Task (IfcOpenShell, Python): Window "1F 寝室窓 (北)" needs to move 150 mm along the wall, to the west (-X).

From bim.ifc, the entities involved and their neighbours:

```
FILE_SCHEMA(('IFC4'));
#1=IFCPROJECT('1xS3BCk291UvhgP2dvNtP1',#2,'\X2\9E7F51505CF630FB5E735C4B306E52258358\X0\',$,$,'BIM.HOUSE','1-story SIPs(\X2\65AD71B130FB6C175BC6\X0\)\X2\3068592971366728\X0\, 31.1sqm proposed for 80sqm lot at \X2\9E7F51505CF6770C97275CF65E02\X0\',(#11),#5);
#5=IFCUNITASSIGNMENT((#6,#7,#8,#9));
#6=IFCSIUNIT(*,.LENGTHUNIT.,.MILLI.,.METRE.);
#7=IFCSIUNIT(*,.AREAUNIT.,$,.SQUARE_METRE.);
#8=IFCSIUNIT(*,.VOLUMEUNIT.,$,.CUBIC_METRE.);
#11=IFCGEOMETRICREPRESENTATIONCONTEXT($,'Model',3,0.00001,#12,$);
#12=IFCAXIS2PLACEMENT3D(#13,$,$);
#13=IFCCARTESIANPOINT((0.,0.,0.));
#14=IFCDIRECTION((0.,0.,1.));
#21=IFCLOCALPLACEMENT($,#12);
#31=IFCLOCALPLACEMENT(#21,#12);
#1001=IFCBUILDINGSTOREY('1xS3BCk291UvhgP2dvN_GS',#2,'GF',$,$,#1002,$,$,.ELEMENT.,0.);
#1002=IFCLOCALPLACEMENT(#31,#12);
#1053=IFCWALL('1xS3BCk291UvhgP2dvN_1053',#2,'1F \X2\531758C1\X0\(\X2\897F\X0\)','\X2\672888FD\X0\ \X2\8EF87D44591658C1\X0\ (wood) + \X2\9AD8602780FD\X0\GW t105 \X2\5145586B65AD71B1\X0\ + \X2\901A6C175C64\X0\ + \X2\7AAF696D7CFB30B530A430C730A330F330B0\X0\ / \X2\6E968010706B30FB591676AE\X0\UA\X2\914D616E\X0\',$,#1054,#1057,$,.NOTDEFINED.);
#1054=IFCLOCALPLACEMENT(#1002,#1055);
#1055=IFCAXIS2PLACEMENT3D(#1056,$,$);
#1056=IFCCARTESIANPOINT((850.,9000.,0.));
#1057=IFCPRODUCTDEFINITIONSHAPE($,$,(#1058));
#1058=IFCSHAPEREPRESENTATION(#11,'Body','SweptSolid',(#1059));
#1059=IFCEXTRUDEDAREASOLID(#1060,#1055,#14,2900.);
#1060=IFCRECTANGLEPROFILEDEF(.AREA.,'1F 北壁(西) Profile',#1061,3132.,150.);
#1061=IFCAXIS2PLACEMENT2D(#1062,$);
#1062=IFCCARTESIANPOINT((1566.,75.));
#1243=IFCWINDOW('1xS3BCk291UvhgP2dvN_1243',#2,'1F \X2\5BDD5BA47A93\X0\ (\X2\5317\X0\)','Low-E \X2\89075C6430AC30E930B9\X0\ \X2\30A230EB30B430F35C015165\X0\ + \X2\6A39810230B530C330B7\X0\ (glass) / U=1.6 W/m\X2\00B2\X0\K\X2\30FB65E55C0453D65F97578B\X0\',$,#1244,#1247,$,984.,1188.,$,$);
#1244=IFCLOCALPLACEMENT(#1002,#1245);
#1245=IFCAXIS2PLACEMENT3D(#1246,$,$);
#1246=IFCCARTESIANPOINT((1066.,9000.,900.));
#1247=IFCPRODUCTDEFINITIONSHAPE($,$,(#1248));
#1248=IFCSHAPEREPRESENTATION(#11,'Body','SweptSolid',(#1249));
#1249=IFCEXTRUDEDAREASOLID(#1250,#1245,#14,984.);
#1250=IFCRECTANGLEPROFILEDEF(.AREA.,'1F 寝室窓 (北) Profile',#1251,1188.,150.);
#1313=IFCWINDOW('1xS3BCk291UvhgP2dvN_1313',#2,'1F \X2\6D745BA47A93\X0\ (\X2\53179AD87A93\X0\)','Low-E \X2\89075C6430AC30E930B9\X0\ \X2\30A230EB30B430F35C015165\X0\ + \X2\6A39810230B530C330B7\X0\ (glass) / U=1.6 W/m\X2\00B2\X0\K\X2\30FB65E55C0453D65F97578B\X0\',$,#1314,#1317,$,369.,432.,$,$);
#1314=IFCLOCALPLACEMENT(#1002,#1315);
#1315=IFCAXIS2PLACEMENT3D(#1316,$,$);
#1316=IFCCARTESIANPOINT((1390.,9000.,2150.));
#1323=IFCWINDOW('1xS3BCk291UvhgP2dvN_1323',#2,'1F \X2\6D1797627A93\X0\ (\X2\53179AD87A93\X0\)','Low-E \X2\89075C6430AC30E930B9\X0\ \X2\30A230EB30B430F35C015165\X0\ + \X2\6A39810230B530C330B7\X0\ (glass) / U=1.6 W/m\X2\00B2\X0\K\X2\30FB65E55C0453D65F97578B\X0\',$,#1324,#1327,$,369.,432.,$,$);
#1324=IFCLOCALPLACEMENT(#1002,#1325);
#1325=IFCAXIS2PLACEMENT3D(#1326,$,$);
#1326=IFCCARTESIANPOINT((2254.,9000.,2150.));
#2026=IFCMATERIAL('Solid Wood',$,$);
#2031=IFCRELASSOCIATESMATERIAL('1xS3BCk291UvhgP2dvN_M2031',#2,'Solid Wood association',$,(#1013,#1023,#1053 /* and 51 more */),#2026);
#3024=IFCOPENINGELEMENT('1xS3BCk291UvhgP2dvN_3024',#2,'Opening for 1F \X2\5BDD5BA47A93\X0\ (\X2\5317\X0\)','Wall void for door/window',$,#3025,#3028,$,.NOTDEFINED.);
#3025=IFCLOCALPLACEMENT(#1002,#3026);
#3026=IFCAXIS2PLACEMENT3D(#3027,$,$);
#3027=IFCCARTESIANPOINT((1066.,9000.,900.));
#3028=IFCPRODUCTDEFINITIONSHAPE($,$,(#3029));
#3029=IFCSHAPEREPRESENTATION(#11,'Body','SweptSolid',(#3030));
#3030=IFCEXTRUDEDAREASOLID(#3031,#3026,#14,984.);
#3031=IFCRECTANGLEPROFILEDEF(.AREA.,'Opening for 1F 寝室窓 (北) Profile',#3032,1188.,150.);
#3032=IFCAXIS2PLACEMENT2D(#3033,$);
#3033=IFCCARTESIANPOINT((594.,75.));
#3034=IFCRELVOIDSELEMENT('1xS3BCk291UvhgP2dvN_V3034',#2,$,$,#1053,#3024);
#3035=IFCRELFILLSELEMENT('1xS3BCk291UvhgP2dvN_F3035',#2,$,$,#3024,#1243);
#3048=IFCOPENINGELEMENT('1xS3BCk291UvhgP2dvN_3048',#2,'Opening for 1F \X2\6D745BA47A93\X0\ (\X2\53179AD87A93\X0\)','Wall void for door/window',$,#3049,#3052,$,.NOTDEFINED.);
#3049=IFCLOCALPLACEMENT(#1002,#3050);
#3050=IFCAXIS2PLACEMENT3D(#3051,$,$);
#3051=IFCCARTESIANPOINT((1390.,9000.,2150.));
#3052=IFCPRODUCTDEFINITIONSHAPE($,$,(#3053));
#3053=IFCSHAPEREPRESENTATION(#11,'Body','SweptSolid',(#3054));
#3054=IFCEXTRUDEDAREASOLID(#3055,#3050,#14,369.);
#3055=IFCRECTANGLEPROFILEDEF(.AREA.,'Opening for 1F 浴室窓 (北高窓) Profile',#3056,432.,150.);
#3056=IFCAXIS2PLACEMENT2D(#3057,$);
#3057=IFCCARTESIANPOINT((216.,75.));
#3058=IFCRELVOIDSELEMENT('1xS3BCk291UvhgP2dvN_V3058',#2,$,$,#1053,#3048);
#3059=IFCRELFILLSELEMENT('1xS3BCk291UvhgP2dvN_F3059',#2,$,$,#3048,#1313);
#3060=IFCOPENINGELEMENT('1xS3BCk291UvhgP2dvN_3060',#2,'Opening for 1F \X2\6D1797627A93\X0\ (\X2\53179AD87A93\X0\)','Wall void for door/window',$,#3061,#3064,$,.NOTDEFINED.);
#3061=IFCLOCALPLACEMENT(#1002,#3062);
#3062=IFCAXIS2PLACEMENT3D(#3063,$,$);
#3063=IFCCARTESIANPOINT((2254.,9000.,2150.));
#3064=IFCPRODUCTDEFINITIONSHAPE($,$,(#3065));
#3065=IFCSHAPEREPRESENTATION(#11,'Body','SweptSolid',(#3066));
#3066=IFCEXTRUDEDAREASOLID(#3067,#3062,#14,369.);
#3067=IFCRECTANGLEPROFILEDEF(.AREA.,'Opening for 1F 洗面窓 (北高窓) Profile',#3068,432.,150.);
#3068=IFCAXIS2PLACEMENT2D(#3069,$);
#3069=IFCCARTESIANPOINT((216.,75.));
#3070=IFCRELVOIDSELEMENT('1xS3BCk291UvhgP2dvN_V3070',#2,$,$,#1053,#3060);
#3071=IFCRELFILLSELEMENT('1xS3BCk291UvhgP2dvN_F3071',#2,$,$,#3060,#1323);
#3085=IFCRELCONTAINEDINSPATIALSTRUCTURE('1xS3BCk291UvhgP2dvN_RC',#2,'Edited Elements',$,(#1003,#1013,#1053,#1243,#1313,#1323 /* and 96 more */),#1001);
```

```python
import ifcopenshell
import ifcopenshell.api.geometry
import ifcopenshell.util.placement
import ifcopenshell.util.unit

model = ifcopenshell.open("bim.ifc")
unit_scale = ifcopenshell.util.unit.calculate_unit_scale(model)

window = model.by_id(1243)
opening = window.FillsVoids[0].RelatingOpeningElement
wall = opening.VoidsElements[0].RelatingBuildingElement

wall_matrix = ifcopenshell.util.placement.get_local_placement(wall.ObjectPlacement)
shift = wall_matrix[:3, 0] * -0.15 / unit_scale
before = ifcopenshell.util.placement.get_local_placement(window.ObjectPlacement)[:3, 3].copy()

# The window is not placed relative to its opening, so move both.
for product in (opening, window):
    matrix = ifcopenshell.util.placement.get_local_placement(product.ObjectPlacement)
    matrix[:3, 3] += shift
    ifcopenshell.api.geometry.edit_object_placement(model, product=product, matrix=matrix, is_si=False)

after = ifcopenshell.util.placement.get_local_placement(window.ObjectPlacement)[:3, 3]
print("window moved by", (after - before).round(3) + 0.0)

model.write("bim_rev.ifc")
```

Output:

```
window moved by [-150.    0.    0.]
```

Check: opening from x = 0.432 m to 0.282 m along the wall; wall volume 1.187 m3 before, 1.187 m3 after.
